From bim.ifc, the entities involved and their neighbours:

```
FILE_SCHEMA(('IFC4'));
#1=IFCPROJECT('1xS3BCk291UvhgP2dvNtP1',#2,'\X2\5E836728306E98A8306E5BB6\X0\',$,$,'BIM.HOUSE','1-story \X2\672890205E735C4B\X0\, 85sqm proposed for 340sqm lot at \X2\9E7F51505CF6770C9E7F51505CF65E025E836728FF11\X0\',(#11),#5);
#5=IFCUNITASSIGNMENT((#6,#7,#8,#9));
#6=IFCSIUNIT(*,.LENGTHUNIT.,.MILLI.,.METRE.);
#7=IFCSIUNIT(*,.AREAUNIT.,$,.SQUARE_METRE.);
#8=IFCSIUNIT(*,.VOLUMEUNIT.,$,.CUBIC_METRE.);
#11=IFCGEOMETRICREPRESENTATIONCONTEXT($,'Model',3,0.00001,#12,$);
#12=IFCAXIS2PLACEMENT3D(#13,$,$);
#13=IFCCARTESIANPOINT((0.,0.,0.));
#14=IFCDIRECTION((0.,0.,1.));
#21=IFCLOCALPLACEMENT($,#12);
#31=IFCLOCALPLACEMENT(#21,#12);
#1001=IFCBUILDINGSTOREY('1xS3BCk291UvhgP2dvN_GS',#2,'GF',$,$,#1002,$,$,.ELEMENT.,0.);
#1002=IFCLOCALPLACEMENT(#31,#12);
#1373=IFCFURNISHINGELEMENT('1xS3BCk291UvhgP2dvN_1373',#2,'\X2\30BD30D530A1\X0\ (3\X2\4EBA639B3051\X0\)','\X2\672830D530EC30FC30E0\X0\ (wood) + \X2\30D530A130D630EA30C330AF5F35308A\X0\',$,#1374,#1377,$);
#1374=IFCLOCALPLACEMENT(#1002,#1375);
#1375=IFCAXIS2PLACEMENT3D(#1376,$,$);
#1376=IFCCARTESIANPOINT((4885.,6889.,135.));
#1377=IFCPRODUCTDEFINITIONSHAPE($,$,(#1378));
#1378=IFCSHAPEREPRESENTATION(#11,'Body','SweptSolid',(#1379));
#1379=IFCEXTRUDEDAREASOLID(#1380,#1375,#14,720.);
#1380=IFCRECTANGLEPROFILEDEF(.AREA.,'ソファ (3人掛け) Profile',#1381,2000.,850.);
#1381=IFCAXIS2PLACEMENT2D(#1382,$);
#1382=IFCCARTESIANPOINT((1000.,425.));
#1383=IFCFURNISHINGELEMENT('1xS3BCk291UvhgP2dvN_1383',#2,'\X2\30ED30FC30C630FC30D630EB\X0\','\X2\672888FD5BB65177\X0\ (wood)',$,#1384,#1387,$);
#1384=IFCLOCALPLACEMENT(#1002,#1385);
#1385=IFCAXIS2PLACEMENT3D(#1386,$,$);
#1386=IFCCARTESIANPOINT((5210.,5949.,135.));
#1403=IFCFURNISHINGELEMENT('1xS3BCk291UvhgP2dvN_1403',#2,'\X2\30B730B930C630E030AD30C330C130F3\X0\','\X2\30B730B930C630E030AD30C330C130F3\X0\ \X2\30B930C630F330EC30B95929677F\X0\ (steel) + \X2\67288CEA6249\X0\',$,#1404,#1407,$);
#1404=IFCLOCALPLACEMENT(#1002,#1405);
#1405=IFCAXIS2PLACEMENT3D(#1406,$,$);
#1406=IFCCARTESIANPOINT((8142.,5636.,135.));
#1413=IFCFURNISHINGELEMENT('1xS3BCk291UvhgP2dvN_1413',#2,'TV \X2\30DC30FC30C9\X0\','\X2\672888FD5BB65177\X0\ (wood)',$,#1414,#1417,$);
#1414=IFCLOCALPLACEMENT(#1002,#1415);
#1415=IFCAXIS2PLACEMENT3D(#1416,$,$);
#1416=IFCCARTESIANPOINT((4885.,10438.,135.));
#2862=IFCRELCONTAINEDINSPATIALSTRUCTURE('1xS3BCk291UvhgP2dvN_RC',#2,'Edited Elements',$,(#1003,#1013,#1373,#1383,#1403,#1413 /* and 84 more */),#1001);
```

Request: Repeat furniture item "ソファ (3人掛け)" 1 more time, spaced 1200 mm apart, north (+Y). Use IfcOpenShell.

```python
import numpy as np
import ifcopenshell
import ifcopenshell.api.geometry
import ifcopenshell.api.root
import ifcopenshell.util.element
import ifcopenshell.util.placement
import ifcopenshell.util.unit

model = ifcopenshell.open("bim.ifc")
unit_scale = ifcopenshell.util.unit.calculate_unit_scale(model)


def reuse_history(source, copy):
    """copy_class also copies each property set's owner history, people and application; keep the originals."""
    for rel in copy.IsDefinedBy:
        if rel.is_a("IfcRelDefinesByProperties") and (history := rel.RelatingPropertyDefinition.OwnerHistory):
            rel.RelatingPropertyDefinition.OwnerHistory = source.OwnerHistory
            ifcopenshell.util.element.remove_deep2(model, history)


source = model.by_guid("1xS3BCk291UvhgP2dvN_1373")
base = ifcopenshell.util.placement.get_local_placement(source.ObjectPlacement)
step = np.array([0.0, 1.0, 0.0]) * 1.2 / unit_scale

for i in range(1, 2):
    copy = ifcopenshell.api.root.copy_class(model, product=source)
    copy.Representation = ifcopenshell.util.element.copy_deep(
        model, source.Representation, exclude=["IfcGeometricRepresentationContext", "IfcRepresentationMap"]
    )
    reuse_history(source, copy)
    matrix = base.copy()
    matrix[:3, 3] += i * step
    print("added at", matrix[:3, 3].round(3) + 0.0)
    ifcopenshell.api.geometry.edit_object_placement(model, product=copy, matrix=matrix, is_si=False)

model.write("bim-out.ifc")
```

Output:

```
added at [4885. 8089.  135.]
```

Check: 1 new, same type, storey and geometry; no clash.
